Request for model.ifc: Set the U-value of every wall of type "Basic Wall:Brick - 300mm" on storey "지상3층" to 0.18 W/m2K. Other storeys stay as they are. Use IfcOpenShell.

First a look at what the model holds.

```python
import ifcopenshell
import ifcopenshell.util.element

model = ifcopenshell.open("model.ifc")
print(model.schema)
storey = next(s for s in model.by_type("IfcBuildingStorey") if s.Name == "지상3층")
walls = [e for e in ifcopenshell.util.element.get_decomposition(storey) if e.is_a("IfcWall")]
seen = {}
for e in walls:
    element_type = ifcopenshell.util.element.get_type(e)
    key = (element_type.Name if element_type != e and element_type else None, ifcopenshell.util.element.get_pset(e, "Pset_WallCommon", "ThermalTransmittance"))
    seen[key] = seen.get(key, 0) + 1
for (name, value), count in sorted(seen.items(), key=str):
    print(count, "x", name, "|", value)
```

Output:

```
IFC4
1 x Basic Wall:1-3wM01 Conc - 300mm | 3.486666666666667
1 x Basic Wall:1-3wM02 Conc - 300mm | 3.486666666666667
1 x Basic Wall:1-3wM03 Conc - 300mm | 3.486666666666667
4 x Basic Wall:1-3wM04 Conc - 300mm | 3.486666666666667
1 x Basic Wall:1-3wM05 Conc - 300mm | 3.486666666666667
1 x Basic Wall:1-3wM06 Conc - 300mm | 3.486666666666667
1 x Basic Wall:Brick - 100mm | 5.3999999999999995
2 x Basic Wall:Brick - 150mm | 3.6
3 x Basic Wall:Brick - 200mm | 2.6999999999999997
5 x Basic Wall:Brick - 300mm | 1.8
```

```python
import ifcopenshell
import ifcopenshell.api.pset
import ifcopenshell.util.element

model = ifcopenshell.open("model.ifc")

storey = next(s for s in model.by_type("IfcBuildingStorey") if s.Name == "지상3층")
walls = [e for e in ifcopenshell.util.element.get_decomposition(storey) if e.is_a("IfcWall")]

count = 0
for e in walls:
    element_type = ifcopenshell.util.element.get_type(e)
    if element_type in (None, e) or element_type.Name != "Basic Wall:Brick - 300mm":
        continue
    # add_pset returns the element's existing set when there is one.
    pset = ifcopenshell.api.pset.add_pset(model, product=e, name="Pset_WallCommon")
    ifcopenshell.api.pset.edit_pset(model, pset=pset, properties={"ThermalTransmittance": 0.18})
    count += 1

print(count, "walls updated")

model.write("model_v2.ifc")
```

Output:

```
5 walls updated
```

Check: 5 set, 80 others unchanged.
